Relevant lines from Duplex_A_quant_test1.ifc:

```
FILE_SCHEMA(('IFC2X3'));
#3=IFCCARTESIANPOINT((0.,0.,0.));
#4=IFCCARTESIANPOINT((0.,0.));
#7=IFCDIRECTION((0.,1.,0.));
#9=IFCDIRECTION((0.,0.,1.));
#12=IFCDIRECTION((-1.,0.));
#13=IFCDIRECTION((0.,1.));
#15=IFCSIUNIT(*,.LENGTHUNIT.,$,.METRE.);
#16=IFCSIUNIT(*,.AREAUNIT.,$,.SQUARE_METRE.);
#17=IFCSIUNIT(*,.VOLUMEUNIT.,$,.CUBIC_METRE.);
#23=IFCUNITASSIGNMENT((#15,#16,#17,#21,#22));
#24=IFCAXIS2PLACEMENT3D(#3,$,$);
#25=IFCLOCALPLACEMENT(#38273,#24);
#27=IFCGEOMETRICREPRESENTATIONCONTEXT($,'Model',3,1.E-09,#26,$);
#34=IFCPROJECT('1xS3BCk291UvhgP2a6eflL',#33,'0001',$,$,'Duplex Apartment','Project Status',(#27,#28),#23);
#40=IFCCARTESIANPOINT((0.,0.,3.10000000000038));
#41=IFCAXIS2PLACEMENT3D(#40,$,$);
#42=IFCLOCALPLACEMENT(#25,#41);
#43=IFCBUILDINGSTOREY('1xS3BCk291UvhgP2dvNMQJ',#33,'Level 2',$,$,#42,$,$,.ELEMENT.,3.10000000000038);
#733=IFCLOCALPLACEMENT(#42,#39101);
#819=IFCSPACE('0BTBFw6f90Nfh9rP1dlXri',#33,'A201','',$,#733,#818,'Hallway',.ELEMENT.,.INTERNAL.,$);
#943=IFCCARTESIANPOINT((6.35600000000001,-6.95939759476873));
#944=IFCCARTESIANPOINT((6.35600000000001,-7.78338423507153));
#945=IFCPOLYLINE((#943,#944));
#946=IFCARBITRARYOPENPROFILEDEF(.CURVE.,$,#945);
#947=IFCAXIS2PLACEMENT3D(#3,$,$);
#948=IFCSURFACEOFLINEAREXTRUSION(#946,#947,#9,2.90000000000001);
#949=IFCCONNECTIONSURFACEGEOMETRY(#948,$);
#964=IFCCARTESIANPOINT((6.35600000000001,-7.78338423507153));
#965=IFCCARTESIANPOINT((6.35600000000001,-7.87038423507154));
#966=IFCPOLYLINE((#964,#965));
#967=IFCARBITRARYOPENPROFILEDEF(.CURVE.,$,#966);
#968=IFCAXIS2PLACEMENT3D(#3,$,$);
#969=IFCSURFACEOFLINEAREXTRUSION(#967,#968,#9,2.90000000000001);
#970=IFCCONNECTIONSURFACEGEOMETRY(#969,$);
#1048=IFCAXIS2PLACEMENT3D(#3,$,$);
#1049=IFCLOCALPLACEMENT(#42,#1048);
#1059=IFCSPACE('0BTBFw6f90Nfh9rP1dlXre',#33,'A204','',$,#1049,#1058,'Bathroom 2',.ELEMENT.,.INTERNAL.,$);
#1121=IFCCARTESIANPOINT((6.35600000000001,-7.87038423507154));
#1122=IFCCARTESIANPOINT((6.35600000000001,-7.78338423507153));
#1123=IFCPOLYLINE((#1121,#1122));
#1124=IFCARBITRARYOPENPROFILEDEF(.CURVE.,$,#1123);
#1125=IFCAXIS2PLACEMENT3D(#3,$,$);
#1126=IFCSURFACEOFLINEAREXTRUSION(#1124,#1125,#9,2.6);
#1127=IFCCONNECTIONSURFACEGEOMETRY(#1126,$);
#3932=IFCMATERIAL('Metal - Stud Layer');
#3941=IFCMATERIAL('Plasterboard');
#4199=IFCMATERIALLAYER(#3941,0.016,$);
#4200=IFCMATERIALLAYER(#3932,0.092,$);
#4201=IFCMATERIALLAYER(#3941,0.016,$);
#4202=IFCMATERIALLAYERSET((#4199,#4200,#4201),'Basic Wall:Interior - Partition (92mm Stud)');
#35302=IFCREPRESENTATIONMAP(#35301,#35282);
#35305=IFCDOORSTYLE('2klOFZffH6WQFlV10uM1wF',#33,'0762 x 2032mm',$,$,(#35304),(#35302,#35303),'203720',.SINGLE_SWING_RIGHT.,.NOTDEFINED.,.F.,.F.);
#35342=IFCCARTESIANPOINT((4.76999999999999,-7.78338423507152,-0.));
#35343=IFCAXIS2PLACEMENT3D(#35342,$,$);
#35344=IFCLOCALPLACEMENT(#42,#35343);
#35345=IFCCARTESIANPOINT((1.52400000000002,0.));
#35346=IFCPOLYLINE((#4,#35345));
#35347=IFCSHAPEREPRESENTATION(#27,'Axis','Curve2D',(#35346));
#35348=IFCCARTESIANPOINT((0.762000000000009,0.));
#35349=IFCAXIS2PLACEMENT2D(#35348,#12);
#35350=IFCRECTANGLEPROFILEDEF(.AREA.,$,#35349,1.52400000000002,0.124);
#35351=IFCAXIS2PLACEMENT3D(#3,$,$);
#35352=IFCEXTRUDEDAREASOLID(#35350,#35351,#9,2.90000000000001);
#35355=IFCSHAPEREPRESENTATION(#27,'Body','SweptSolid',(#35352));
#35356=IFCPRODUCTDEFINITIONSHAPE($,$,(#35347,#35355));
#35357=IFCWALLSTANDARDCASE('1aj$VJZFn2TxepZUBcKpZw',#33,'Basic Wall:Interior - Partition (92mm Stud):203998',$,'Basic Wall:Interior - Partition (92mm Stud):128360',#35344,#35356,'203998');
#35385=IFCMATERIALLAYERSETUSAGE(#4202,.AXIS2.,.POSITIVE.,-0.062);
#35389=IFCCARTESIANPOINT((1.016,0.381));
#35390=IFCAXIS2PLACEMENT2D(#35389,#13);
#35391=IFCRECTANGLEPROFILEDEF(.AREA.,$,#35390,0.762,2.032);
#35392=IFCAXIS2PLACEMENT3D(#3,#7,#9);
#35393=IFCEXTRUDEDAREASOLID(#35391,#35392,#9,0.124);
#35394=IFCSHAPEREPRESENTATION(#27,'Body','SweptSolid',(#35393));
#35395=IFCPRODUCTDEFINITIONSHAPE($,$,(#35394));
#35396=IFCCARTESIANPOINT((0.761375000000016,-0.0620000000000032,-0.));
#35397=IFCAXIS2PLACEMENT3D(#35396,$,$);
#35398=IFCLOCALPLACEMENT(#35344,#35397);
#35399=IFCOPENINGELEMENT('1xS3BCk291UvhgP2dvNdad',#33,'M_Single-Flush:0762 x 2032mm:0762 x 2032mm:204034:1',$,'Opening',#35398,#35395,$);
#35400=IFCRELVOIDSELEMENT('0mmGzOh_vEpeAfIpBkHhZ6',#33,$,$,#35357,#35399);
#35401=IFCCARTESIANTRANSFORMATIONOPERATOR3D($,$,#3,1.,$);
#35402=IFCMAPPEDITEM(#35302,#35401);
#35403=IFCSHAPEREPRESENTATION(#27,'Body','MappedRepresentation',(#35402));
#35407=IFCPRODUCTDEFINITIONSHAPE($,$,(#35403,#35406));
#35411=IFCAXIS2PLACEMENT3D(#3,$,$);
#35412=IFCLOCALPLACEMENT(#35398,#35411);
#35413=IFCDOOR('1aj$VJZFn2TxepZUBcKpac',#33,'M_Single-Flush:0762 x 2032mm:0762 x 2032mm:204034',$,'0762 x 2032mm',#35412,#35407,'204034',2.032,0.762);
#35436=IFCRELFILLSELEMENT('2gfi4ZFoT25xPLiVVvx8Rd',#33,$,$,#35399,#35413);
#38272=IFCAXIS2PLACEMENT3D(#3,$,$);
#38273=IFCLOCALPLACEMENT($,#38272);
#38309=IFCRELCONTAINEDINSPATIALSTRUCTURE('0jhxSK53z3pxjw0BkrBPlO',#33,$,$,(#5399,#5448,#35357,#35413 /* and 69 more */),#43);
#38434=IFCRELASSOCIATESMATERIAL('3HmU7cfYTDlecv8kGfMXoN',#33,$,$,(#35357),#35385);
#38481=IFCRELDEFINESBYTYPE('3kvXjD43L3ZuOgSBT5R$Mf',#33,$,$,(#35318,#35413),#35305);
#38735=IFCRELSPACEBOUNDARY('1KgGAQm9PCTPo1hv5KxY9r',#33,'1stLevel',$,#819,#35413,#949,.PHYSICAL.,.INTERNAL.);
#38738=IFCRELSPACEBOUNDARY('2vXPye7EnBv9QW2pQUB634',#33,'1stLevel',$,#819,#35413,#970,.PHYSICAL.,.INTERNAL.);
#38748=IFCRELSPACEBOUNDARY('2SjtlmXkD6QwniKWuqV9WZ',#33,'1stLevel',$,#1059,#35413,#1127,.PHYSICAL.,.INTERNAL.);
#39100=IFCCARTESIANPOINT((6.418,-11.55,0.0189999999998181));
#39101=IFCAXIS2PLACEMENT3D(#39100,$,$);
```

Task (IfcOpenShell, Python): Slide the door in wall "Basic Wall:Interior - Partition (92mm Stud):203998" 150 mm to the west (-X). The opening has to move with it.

```python
import numpy as np
import ifcopenshell
import ifcopenshell.api.geometry
import ifcopenshell.util.placement
import ifcopenshell.util.unit

model = ifcopenshell.open("Duplex_A_quant_test1.ifc")
unit_scale = ifcopenshell.util.unit.calculate_unit_scale(model)

door = model.by_guid("1aj$VJZFn2TxepZUBcKpac")
opening = door.FillsVoids[0].RelatingOpeningElement
wall = opening.VoidsElements[0].RelatingBuildingElement

wall_matrix = ifcopenshell.util.placement.get_local_placement(wall.ObjectPlacement)
shift = wall_matrix[:3, 0] * -0.15 / unit_scale
before = ifcopenshell.util.placement.get_local_placement(door.ObjectPlacement)[:3, 3].copy()

# The door is placed relative to its opening, so it follows when the opening moves.
matrix = ifcopenshell.util.placement.get_local_placement(opening.ObjectPlacement)
matrix[:3, 3] += shift
ifcopenshell.api.geometry.edit_object_placement(
    model, product=opening, matrix=matrix, is_si=False, should_transform_children=True
)

# Space boundary surfaces are stored in each space's coordinates; move them too.
for rel in door.ProvidesBoundaries:
    if not rel.ConnectionGeometry:
        continue
    surface = rel.ConnectionGeometry.SurfaceOnRelatingElement
    space_matrix = ifcopenshell.util.placement.get_local_placement(rel.RelatingSpace.ObjectPlacement)
    point = np.array(surface.Position.Location.Coordinates) + space_matrix[:3, :3].T @ shift
    surface.Position = model.createIfcAxis2Placement3D(
        model.createIfcCartesianPoint(point.tolist()), surface.Position.Axis, surface.Position.RefDirection
    )

after = ifcopenshell.util.placement.get_local_placement(door.ObjectPlacement)[:3, 3]
print("door moved by", (after - before).round(3) + 0.0)

model.write("Duplex_A_quant_test1-out.ifc")
```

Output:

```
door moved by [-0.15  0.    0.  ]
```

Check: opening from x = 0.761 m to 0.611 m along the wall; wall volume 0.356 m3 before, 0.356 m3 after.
